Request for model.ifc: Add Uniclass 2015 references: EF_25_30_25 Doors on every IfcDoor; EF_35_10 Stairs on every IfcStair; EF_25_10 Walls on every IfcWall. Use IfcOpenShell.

First a look at what the model holds.

```python
import ifcopenshell

model = ifcopenshell.open("model.ifc")
print(model.schema)
print("classifications:", [c.Name for c in model.by_type("IfcClassification")])
for ifc_class in ("IfcDoor", "IfcRoof", "IfcStair", "IfcWall", "IfcWindow"):
    print(ifc_class, len(model.by_type(ifc_class)))
```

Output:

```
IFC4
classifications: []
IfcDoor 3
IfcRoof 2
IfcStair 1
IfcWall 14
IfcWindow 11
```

```python
import ifcopenshell
import ifcopenshell.api.classification

model = ifcopenshell.open("model.ifc")

system = ifcopenshell.api.classification.add_classification(model, classification="Uniclass 2015")

codes = {
    "IfcDoor": ("EF_25_30_25", "Doors"),
    "IfcStair": ("EF_35_10", "Stairs"),
    "IfcWall": ("EF_25_10", "Walls"),
}
for ifc_class, (code, name) in codes.items():
    products = model.by_type(ifc_class)
    ifcopenshell.api.classification.add_reference(
        model, products=products, classification=system, identification=code, name=name
    )
    print(code, len(products))

model.write("model_edited.ifc")
```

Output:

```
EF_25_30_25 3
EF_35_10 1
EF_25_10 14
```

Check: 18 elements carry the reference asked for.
